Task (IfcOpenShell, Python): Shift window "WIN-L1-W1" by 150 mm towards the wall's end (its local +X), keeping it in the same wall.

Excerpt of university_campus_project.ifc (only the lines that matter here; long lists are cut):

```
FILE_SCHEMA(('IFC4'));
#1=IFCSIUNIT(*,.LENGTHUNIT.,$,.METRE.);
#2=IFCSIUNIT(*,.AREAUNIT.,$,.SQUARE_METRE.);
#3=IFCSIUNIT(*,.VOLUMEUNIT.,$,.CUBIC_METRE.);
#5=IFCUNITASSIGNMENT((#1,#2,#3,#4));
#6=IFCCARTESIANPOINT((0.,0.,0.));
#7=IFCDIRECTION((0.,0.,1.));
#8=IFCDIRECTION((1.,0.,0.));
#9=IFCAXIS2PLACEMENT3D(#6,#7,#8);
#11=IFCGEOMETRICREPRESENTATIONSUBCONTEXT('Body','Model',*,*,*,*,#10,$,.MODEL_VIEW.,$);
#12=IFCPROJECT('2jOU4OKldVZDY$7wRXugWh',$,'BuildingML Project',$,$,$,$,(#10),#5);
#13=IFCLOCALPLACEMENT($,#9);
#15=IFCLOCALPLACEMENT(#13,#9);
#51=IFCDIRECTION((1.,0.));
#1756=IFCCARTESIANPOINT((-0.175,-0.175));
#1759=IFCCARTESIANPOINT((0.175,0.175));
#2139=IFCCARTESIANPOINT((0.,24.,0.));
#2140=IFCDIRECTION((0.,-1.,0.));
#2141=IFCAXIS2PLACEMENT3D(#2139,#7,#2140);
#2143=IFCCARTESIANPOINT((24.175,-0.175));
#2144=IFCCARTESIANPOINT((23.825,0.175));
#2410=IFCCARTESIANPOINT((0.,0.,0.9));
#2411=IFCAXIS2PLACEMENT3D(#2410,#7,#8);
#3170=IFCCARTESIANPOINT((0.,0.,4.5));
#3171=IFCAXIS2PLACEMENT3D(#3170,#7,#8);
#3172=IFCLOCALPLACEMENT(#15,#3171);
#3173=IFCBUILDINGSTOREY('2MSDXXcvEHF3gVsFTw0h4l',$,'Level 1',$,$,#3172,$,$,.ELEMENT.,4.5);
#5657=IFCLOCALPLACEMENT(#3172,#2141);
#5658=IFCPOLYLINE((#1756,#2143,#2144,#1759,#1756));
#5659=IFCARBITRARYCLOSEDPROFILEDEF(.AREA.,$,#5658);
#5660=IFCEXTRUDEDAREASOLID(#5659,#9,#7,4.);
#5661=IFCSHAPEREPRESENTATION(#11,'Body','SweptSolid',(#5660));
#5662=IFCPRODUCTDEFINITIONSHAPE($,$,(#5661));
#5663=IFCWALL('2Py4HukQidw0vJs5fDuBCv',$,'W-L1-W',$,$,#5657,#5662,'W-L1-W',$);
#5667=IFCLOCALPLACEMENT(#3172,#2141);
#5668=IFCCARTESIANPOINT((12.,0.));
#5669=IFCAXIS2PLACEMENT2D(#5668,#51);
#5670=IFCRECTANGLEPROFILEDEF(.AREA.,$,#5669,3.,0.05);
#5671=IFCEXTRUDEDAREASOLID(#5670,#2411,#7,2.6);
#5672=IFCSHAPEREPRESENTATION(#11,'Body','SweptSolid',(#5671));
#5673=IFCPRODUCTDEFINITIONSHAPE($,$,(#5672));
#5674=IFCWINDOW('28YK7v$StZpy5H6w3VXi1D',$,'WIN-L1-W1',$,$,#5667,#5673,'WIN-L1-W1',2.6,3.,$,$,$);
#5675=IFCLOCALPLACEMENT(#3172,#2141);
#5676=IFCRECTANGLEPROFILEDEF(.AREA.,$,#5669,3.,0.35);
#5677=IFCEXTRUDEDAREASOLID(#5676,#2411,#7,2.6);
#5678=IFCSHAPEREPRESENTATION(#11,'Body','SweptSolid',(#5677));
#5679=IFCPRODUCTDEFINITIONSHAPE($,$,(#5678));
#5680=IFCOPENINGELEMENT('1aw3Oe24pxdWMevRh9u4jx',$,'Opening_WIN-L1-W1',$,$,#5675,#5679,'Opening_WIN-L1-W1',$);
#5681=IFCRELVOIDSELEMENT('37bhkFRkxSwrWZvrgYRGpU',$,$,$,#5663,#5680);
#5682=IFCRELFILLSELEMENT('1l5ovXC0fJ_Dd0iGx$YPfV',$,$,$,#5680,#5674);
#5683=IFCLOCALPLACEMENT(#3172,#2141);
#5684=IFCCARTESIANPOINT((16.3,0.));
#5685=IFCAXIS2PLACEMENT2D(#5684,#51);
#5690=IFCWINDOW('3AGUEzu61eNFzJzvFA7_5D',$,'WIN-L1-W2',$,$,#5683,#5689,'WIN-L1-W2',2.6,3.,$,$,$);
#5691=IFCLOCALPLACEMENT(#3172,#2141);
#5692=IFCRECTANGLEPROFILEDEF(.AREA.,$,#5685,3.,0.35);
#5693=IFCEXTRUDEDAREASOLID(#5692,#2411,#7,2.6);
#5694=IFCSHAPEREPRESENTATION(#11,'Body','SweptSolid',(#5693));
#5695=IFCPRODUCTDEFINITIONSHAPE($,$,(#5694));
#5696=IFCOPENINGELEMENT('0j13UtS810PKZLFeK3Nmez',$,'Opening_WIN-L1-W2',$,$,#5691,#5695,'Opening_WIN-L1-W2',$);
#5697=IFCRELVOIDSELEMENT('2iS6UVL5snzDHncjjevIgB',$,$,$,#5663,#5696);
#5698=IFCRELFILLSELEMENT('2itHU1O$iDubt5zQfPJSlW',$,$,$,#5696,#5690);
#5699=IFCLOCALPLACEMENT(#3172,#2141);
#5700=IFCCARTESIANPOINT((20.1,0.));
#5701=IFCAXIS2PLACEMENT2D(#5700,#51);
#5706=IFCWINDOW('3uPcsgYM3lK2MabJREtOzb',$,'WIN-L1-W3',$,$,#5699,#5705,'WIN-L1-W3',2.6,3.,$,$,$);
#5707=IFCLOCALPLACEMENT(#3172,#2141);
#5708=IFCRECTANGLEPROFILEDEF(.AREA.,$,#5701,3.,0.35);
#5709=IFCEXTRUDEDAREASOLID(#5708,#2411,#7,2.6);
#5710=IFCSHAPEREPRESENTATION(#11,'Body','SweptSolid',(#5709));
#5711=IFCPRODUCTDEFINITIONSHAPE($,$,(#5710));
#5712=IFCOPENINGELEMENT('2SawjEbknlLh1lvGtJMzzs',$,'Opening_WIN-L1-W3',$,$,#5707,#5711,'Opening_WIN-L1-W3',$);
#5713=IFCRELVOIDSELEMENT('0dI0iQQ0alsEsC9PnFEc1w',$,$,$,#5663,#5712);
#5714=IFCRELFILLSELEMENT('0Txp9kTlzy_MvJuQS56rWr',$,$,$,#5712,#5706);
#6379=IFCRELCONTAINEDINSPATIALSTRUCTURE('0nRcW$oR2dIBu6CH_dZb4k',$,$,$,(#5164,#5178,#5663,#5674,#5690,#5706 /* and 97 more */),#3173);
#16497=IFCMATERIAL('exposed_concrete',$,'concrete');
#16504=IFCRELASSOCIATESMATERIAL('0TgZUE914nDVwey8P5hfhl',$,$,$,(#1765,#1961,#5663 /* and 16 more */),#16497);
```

```python
import ifcopenshell
import ifcopenshell.api.geometry
import ifcopenshell.util.placement
import ifcopenshell.util.unit

model = ifcopenshell.open("university_campus_project.ifc")
unit_scale = ifcopenshell.util.unit.calculate_unit_scale(model)

window = model.by_guid("28YK7v$StZpy5H6w3VXi1D")
opening = window.FillsVoids[0].RelatingOpeningElement
wall = opening.VoidsElements[0].RelatingBuildingElement

wall_matrix = ifcopenshell.util.placement.get_local_placement(wall.ObjectPlacement)
shift = wall_matrix[:3, 0] * 0.15 / unit_scale
before = ifcopenshell.util.placement.get_local_placement(window.ObjectPlacement)[:3, 3].copy()

# The window is not placed relative to its opening, so move both.
for product in (opening, window):
    matrix = ifcopenshell.util.placement.get_local_placement(product.ObjectPlacement)
    matrix[:3, 3] += shift
    ifcopenshell.api.geometry.edit_object_placement(model, product=product, matrix=matrix, is_si=False)

after = ifcopenshell.util.placement.get_local_placement(window.ObjectPlacement)[:3, 3]
print("window moved by", (after - before).round(3) + 0.0)

model.write("university_campus_project_rev.ifc")
```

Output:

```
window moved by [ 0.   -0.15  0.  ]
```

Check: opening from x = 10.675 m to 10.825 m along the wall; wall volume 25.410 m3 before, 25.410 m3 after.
